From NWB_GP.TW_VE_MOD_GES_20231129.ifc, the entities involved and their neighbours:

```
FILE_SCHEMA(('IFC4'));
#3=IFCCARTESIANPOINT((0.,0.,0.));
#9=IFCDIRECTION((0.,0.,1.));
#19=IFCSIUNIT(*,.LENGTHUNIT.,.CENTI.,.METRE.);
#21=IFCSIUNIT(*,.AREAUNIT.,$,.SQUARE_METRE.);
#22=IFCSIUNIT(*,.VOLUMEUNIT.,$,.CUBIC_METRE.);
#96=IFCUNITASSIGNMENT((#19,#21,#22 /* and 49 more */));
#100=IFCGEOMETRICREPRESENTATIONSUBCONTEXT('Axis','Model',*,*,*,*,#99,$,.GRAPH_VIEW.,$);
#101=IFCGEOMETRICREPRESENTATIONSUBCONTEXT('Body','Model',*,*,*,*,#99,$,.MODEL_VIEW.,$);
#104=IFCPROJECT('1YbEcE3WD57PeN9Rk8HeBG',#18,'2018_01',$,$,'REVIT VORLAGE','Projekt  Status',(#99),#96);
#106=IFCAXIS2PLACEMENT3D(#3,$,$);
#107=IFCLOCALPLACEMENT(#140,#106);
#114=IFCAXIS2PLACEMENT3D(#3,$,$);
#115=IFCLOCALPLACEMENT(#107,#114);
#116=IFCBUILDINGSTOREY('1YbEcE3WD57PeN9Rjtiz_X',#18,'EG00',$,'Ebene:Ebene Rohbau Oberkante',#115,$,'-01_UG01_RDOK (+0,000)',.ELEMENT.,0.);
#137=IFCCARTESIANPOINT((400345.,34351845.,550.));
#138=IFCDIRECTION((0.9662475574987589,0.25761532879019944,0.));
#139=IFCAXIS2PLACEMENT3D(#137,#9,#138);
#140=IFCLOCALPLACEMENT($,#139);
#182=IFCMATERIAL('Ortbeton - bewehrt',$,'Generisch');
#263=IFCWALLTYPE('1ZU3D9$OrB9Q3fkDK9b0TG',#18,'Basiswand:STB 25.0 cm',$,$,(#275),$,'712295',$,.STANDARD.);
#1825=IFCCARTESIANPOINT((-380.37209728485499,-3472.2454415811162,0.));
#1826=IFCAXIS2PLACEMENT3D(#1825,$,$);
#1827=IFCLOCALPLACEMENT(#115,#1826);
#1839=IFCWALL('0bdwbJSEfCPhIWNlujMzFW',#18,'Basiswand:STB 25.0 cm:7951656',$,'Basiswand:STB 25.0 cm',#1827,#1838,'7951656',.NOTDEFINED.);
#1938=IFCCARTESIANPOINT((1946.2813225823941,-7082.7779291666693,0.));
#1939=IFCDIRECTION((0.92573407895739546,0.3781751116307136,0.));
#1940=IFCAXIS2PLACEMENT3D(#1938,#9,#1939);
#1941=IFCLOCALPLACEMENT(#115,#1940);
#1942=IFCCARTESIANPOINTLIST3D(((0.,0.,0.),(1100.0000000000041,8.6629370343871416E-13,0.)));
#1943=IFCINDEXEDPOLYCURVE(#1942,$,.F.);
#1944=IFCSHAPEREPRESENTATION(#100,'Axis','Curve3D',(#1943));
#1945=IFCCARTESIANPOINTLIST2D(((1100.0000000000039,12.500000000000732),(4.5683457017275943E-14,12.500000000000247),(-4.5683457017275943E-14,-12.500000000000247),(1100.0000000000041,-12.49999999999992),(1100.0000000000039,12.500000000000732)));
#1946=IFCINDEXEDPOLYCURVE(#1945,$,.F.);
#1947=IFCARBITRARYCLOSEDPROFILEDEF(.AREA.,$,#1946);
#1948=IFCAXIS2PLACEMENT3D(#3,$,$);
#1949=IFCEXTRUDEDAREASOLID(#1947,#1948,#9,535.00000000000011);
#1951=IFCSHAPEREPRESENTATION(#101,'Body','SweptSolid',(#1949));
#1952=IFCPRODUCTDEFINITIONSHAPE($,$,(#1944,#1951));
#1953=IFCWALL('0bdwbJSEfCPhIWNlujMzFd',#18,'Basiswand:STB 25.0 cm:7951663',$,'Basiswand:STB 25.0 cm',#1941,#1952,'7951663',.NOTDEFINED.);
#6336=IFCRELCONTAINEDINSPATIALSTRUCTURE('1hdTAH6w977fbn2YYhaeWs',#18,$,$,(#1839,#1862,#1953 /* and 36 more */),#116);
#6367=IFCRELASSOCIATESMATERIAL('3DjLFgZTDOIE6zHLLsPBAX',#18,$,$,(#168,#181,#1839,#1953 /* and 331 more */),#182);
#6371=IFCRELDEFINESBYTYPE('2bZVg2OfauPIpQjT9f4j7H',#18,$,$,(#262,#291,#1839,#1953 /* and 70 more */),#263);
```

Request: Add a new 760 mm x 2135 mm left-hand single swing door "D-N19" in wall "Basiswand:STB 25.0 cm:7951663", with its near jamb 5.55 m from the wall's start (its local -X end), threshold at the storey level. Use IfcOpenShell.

```python
import numpy as np
import ifcopenshell
import ifcopenshell.api.feature
import ifcopenshell.api.geometry
import ifcopenshell.api.root
import ifcopenshell.api.spatial
import ifcopenshell.geom
import ifcopenshell.util.element
import ifcopenshell.util.placement
import ifcopenshell.util.representation
import ifcopenshell.util.shape
import ifcopenshell.util.unit

model = ifcopenshell.open("NWB_GP.TW_VE_MOD_GES_20231129.ifc")
unit_scale = ifcopenshell.util.unit.calculate_unit_scale(model)
settings = ifcopenshell.geom.settings()


def volume(element):
    """Net volume in cubic metres, openings subtracted."""
    shape = ifcopenshell.geom.create_shape(settings, element)
    return ifcopenshell.util.shape.get_volume(shape.geometry)


wall = model.by_guid("0bdwbJSEfCPhIWNlujMzFd")
storey = ifcopenshell.util.element.get_container(wall, ifc_class="IfcBuildingStorey")
context = ifcopenshell.util.representation.get_context(model, "Model", "Body", "MODEL_VIEW")
before = volume(wall)

width, height, from_end, sill = 0.76, 2.135, 5.55, 0.0  # metres

# The wall runs along its own X axis, and the end named is its -X end.
wall_shape = ifcopenshell.geom.create_shape(settings, wall)
x, y, z = ifcopenshell.util.shape.get_vertices(wall_shape.geometry).T
start = x.min() + from_end
face, thickness = float(y.min()), float(y.max() - y.min())
wall_matrix = ifcopenshell.util.placement.get_local_placement(wall.ObjectPlacement)
level = ifcopenshell.util.placement.get_local_placement(storey.ObjectPlacement)[2, 3]


def in_wall(x, y):
    """Placement at x, y metres in the wall's axes, at sill height."""
    matrix = wall_matrix.copy()
    matrix[:, 3] = wall_matrix @ np.array([x / unit_scale, y / unit_scale, 0.0, 1.0])
    matrix[2, 3] = level + sill / unit_scale
    return matrix


# Opening: a box that overshoots both wall faces by 50 mm.
opening = ifcopenshell.api.root.create_entity(model, ifc_class="IfcOpeningElement", predefined_type="OPENING")
box = ifcopenshell.api.geometry.add_wall_representation(
    model, context=context, length=width, height=height, thickness=thickness + 0.1
)
ifcopenshell.api.geometry.assign_representation(model, product=opening, representation=box)
ifcopenshell.api.geometry.edit_object_placement(model, product=opening, matrix=in_wall(start, face - 0.05), is_si=False)
ifcopenshell.api.feature.add_feature(model, feature=opening, element=wall)

door = ifcopenshell.api.root.create_entity(model, ifc_class="IfcDoor", name="D-N19", predefined_type="DOOR")
door.OverallWidth, door.OverallHeight = width / unit_scale, height / unit_scale
door.OperationType = "SINGLE_SWING_LEFT"
body = ifcopenshell.api.geometry.add_door_representation(
    model,
    context=context,
    overall_width=door.OverallWidth,
    overall_height=door.OverallHeight,
    operation_type="SINGLE_SWING_LEFT",
    lining_properties={"LiningDepth": thickness / unit_scale, "ThresholdDepth": thickness / unit_scale},
)
ifcopenshell.api.geometry.assign_representation(model, product=door, representation=body)
ifcopenshell.api.spatial.assign_container(model, products=[door], relating_structure=storey)
ifcopenshell.api.feature.add_filling(model, opening=opening, element=door)

# The lining spans the wall, so the door starts at the wall face.
ifcopenshell.api.geometry.edit_object_placement(model, product=door, matrix=in_wall(start, face), is_si=False)

after = volume(wall)

print(f"wall volume {before:.3f} -> {after:.3f} m3")

model.write("NWB_GP.TW_VE_MOD_GES_20231129-out.ifc")
```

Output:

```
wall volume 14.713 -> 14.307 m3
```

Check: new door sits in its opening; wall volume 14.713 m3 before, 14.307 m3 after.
